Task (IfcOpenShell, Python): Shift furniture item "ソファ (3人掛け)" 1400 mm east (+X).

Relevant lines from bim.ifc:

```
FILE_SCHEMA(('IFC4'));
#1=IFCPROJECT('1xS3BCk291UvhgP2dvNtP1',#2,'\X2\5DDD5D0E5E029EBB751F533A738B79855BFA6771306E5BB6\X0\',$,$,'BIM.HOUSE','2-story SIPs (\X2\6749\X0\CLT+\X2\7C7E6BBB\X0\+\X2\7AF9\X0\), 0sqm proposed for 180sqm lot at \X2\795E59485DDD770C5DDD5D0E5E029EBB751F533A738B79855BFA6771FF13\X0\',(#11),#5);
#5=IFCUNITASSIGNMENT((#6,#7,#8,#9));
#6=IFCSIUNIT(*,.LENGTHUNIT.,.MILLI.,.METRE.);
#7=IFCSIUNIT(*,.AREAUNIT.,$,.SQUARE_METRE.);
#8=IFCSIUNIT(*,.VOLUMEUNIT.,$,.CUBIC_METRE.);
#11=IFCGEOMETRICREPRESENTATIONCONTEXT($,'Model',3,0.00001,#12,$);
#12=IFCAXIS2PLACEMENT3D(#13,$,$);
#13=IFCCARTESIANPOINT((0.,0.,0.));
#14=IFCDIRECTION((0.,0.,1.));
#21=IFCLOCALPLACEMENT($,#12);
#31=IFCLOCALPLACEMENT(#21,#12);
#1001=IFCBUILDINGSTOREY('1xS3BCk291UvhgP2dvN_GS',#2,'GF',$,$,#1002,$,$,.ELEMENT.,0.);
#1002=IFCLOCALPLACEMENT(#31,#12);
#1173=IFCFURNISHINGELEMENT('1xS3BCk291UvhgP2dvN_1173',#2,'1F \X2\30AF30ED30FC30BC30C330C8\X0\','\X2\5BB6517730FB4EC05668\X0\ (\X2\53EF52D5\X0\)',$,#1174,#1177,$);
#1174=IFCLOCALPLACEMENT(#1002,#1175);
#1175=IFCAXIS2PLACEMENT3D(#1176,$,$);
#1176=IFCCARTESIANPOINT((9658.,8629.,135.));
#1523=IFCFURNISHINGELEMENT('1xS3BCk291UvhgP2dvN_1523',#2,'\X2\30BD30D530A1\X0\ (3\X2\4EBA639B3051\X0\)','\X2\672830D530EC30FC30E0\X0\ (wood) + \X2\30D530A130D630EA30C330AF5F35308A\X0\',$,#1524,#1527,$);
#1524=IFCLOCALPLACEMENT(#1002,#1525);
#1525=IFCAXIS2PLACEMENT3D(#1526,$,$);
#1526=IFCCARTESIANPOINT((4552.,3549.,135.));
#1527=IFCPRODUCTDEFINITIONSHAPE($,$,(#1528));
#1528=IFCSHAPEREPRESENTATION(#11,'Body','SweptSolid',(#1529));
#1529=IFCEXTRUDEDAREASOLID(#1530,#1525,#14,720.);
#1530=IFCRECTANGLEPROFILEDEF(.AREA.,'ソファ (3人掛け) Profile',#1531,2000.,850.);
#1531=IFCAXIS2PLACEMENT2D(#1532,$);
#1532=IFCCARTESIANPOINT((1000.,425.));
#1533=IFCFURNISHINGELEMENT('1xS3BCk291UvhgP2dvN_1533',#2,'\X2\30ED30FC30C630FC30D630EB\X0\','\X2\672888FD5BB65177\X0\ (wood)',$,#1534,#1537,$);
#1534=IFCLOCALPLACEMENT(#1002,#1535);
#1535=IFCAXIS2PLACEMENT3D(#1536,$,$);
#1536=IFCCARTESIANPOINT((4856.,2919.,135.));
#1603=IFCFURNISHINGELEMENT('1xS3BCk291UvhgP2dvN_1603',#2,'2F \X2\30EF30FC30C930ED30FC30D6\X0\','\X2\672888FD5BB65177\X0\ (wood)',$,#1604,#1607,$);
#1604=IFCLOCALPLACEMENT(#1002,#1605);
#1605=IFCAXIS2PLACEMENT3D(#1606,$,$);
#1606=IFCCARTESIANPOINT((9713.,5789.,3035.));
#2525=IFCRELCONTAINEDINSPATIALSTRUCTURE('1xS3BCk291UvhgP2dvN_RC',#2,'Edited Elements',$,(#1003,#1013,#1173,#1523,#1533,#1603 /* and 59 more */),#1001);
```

```python
import ifcopenshell
import ifcopenshell.api.geometry
import ifcopenshell.util.placement

model = ifcopenshell.open("bim.ifc")

item = model.by_guid("1xS3BCk291UvhgP2dvN_1523")
matrix = ifcopenshell.util.placement.get_local_placement(item.ObjectPlacement)
matrix[0, 3] += 1400.0
ifcopenshell.api.geometry.edit_object_placement(model, product=item, matrix=matrix, is_si=False)

print(ifcopenshell.util.placement.get_local_placement(item.ObjectPlacement).round(3) + 0.0)

model.write("bim_v2.ifc")
```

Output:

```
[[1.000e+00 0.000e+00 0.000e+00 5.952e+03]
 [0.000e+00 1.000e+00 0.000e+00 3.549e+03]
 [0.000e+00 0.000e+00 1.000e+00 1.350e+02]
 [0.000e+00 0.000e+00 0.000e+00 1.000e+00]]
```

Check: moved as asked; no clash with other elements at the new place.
